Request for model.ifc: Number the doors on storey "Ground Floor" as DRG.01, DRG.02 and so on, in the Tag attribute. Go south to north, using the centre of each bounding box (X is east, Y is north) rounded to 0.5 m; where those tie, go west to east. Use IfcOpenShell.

First a look at what the model holds.

```python
import ifcopenshell
import ifcopenshell.util.element
import ifcopenshell.util.placement

model = ifcopenshell.open("model.ifc")
print(model.schema)
storey = next(s for s in model.by_type("IfcBuildingStorey") if s.Name == "Ground Floor")
doors = [e for e in ifcopenshell.util.element.get_decomposition(storey) if e.is_a("IfcDoor")]
for e in sorted(doors, key=lambda e: e.id()):
    origin = ifcopenshell.util.placement.get_local_placement(e.ObjectPlacement)[:3, 3]
    print(e.id(), e.Tag, e.Name, origin.round(2) + 0.0, sep=" | ")
```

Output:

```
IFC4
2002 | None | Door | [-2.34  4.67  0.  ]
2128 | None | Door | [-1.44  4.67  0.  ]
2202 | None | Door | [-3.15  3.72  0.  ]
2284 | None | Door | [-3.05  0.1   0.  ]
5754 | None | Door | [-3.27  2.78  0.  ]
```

```python
import ifcopenshell
import ifcopenshell.geom
import ifcopenshell.util.element
import ifcopenshell.util.shape

model = ifcopenshell.open("model.ifc")
settings = ifcopenshell.geom.settings()
settings.set("use-world-coords", True)


def centre(element):
    shape = ifcopenshell.geom.create_shape(settings, element)
    return ifcopenshell.util.shape.get_bbox_centroid(shape.geometry)


storey = next(s for s in model.by_type("IfcBuildingStorey") if s.Name == "Ground Floor")
doors = [e for e in ifcopenshell.util.element.get_decomposition(storey) if e.is_a("IfcDoor")]

# Insertion points can sit at a corner or the storey origin, so sort by the geometry (in metres).
centres = {e: centre(e) for e in doors}
doors.sort(key=lambda e: (round(centres[e][1] / 0.5), centres[e][0]))

for i, e in enumerate(doors, start=1):
    number = f"DRG.{i:02d}"
    e.Tag = number
    print(e.id(), number)

model.write("model_rev.ifc")
```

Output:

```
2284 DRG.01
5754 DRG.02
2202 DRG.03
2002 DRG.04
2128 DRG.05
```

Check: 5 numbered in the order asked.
